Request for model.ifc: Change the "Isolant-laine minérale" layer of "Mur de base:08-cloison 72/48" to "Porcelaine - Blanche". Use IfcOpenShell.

First a look at what the model holds.

```python
import ifcopenshell
import ifcopenshell.util.element

model = ifcopenshell.open("model.ifc")
print(model.schema)
for layer_set in model.by_type("IfcMaterialLayerSet"):
    if layer_set.LayerSetName == "Mur de base:08-cloison 72/48":
        for layer in layer_set.MaterialLayers:
            print(layer.id(), layer.Material and layer.Material.Name, layer.LayerThickness, sep=" | ")
        print(len(ifcopenshell.util.element.get_elements_by_material(model, layer_set)), "elements and types use it")
print(sorted(m.Name for m in model.by_type("IfcMaterial") if m.Name)[:60])
```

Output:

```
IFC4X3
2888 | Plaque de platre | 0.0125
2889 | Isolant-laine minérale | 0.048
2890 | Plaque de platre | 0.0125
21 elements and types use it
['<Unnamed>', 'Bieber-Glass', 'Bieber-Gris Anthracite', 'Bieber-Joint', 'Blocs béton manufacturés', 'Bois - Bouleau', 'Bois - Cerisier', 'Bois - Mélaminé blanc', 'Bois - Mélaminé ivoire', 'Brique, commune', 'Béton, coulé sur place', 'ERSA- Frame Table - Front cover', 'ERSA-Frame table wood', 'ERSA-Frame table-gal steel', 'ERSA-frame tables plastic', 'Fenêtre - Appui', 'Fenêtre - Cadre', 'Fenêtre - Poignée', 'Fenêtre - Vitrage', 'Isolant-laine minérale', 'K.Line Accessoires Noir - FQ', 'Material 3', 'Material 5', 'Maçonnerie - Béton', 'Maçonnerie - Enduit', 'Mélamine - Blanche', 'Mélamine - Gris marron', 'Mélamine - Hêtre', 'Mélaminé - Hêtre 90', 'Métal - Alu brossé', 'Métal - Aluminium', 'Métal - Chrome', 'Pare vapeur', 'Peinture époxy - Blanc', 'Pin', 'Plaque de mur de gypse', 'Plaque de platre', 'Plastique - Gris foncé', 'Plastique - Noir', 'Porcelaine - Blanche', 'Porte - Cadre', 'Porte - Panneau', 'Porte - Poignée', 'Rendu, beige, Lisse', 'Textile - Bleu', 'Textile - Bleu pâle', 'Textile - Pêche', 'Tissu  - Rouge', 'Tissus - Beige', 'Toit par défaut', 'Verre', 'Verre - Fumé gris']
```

```python
import ifcopenshell
import ifcopenshell.api.material

model = ifcopenshell.open("model.ifc")

layer_set = next(s for s in model.by_type("IfcMaterialLayerSet") if s.LayerSetName == "Mur de base:08-cloison 72/48")
layer = next(l for l in layer_set.MaterialLayers if l.Material and l.Material.Name == "Isolant-laine minérale")
material = next(m for m in model.by_type("IfcMaterial") if m.Name == "Porcelaine - Blanche")

# Point this one layer at the other material; renaming the old one would change it everywhere.
ifcopenshell.api.material.edit_layer(model, layer=layer, attributes={"Name": material.Name}, material=material)

print([l.Material.Name if l.Material else None for l in layer_set.MaterialLayers])

model.write("model-out.ifc")
```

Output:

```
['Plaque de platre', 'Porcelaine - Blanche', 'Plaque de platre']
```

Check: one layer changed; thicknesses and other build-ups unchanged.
